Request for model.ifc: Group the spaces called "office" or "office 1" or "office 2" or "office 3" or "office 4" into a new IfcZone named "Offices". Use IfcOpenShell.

First a look at what the model holds.

```python
import ifcopenshell

model = ifcopenshell.open("model.ifc")
print(model.schema)
seen = {}
for space in model.by_type("IfcSpace"):
    seen[space.LongName] = seen.get(space.LongName, 0) + 1
for name, count in sorted(seen.items(), key=str):
    print(count, "x", name)
print("zones:", [z.Name for z in model.by_type("IfcZone")][:20])
```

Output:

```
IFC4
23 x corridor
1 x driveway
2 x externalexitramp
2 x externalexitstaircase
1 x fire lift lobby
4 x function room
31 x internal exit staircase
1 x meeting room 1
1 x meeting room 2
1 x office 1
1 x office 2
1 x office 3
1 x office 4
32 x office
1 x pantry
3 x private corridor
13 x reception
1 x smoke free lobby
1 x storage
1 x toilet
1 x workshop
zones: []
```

```python
import ifcopenshell
import ifcopenshell.api.group
import ifcopenshell.api.root

model = ifcopenshell.open("model.ifc")

names = {"office", "office 1", "office 2", "office 3", "office 4"}
spaces = [s for s in model.by_type("IfcSpace") if s.LongName in names]

zone = ifcopenshell.api.root.create_entity(model, ifc_class="IfcZone", name="Offices")
ifcopenshell.api.group.assign_group(model, products=spaces, group=zone)
print(len(spaces), "spaces in", zone.Name)

model.write("model_rev.ifc")
```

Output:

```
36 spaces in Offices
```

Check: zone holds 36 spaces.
